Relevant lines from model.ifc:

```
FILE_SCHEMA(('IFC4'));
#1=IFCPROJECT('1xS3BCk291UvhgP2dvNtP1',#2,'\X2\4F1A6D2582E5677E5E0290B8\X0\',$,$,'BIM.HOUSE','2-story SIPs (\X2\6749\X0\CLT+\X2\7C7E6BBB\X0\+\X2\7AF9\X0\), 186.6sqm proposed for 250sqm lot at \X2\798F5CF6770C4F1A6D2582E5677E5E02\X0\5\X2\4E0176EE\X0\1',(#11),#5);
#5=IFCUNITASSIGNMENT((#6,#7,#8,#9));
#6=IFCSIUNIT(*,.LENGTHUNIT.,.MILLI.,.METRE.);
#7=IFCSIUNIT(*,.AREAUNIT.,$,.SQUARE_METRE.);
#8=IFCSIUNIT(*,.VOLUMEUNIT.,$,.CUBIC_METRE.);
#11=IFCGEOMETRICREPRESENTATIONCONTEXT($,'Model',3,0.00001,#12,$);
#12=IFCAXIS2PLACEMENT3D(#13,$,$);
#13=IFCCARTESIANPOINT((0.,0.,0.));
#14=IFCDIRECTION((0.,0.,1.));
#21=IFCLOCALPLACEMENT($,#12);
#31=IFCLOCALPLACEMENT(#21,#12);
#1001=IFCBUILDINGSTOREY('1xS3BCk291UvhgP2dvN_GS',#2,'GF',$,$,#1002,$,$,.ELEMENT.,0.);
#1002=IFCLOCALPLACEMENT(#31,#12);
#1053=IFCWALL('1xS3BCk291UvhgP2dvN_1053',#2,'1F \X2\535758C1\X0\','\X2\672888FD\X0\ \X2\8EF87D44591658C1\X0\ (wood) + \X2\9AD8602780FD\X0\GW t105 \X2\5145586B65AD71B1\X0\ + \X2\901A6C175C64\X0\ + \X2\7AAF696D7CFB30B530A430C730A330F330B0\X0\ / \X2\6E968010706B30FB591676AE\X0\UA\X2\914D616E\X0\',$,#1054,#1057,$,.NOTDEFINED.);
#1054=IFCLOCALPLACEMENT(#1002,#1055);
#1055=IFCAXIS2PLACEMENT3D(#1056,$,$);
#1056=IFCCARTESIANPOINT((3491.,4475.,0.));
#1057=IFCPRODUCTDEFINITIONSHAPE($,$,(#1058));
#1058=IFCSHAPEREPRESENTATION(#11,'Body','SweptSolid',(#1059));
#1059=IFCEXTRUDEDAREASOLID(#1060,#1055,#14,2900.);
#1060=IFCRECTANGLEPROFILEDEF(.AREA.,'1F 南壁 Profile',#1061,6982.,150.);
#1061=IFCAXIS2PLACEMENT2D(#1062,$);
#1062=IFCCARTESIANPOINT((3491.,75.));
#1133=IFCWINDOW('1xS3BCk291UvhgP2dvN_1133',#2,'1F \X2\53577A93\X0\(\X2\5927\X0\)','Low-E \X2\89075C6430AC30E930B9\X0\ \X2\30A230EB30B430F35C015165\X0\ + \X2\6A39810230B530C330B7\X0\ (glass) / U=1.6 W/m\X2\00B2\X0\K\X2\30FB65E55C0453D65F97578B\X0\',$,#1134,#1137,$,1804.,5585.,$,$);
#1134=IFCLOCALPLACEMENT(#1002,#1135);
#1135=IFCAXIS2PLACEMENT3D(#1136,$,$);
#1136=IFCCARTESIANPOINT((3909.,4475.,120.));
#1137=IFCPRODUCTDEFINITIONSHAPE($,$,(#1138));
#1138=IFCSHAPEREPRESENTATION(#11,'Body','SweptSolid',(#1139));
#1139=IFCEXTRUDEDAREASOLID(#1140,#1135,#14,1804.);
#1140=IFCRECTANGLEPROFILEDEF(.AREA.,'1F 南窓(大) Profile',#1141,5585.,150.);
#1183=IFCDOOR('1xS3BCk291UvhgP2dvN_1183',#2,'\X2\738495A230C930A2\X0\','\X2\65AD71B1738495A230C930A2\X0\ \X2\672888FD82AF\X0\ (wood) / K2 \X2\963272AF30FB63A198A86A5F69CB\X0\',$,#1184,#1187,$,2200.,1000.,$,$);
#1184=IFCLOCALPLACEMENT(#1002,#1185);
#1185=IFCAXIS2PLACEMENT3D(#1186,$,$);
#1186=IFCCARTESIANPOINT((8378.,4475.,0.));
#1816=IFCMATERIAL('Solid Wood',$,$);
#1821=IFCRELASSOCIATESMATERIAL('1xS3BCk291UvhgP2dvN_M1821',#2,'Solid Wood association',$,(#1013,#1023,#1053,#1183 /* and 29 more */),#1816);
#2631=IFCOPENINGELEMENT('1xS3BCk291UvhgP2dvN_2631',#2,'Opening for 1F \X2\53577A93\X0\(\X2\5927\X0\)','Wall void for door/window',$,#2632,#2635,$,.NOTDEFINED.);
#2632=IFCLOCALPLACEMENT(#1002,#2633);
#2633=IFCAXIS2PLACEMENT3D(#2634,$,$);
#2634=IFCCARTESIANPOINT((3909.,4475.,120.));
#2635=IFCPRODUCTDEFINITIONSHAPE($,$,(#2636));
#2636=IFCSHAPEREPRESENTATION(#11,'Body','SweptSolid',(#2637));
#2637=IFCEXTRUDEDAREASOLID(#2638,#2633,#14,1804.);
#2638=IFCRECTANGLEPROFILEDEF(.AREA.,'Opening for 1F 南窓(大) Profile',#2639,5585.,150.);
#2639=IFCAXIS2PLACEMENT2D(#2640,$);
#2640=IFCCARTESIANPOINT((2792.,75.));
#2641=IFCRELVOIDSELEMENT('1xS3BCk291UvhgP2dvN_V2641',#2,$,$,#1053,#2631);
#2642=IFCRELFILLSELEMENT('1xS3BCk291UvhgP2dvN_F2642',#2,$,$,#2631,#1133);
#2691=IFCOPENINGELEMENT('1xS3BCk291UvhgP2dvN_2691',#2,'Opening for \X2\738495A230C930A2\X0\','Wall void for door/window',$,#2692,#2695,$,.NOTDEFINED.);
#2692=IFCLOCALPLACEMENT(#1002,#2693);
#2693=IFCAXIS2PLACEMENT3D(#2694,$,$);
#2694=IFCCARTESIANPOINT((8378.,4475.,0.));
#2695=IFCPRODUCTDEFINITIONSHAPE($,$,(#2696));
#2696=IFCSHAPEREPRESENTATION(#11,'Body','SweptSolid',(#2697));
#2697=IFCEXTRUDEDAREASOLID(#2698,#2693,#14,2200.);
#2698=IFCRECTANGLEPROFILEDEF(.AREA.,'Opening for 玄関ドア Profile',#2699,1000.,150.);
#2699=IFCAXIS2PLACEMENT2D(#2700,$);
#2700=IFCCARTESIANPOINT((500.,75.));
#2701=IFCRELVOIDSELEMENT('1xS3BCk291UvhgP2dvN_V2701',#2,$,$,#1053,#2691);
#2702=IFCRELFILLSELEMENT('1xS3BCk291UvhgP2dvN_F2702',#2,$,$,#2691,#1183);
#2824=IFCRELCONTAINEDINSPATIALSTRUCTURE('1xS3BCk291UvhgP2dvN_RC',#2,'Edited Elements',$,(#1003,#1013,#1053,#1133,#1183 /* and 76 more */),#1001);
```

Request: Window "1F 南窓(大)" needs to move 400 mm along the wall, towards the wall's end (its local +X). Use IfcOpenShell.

```python
import ifcopenshell
import ifcopenshell.api.geometry
import ifcopenshell.util.placement

model = ifcopenshell.open("model.ifc")

window = model.by_guid("1xS3BCk291UvhgP2dvN_1133")
opening = window.FillsVoids[0].RelatingOpeningElement
wall = opening.VoidsElements[0].RelatingBuildingElement

wall_matrix = ifcopenshell.util.placement.get_local_placement(wall.ObjectPlacement)
shift = wall_matrix[:3, 0] * 400.0
before = ifcopenshell.util.placement.get_local_placement(window.ObjectPlacement)[:3, 3].copy()

# The window is not placed relative to its opening, so move both.
for product in (opening, window):
    matrix = ifcopenshell.util.placement.get_local_placement(product.ObjectPlacement)
    matrix[:3, 3] += shift
    ifcopenshell.api.geometry.edit_object_placement(model, product=product, matrix=matrix, is_si=False)

after = ifcopenshell.util.placement.get_local_placement(window.ObjectPlacement)[:3, 3]
print("window moved by", (after - before).round(3) + 0.0)

model.write("model_v2.ifc")
```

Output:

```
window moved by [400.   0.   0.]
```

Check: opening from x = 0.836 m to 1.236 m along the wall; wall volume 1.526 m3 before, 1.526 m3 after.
